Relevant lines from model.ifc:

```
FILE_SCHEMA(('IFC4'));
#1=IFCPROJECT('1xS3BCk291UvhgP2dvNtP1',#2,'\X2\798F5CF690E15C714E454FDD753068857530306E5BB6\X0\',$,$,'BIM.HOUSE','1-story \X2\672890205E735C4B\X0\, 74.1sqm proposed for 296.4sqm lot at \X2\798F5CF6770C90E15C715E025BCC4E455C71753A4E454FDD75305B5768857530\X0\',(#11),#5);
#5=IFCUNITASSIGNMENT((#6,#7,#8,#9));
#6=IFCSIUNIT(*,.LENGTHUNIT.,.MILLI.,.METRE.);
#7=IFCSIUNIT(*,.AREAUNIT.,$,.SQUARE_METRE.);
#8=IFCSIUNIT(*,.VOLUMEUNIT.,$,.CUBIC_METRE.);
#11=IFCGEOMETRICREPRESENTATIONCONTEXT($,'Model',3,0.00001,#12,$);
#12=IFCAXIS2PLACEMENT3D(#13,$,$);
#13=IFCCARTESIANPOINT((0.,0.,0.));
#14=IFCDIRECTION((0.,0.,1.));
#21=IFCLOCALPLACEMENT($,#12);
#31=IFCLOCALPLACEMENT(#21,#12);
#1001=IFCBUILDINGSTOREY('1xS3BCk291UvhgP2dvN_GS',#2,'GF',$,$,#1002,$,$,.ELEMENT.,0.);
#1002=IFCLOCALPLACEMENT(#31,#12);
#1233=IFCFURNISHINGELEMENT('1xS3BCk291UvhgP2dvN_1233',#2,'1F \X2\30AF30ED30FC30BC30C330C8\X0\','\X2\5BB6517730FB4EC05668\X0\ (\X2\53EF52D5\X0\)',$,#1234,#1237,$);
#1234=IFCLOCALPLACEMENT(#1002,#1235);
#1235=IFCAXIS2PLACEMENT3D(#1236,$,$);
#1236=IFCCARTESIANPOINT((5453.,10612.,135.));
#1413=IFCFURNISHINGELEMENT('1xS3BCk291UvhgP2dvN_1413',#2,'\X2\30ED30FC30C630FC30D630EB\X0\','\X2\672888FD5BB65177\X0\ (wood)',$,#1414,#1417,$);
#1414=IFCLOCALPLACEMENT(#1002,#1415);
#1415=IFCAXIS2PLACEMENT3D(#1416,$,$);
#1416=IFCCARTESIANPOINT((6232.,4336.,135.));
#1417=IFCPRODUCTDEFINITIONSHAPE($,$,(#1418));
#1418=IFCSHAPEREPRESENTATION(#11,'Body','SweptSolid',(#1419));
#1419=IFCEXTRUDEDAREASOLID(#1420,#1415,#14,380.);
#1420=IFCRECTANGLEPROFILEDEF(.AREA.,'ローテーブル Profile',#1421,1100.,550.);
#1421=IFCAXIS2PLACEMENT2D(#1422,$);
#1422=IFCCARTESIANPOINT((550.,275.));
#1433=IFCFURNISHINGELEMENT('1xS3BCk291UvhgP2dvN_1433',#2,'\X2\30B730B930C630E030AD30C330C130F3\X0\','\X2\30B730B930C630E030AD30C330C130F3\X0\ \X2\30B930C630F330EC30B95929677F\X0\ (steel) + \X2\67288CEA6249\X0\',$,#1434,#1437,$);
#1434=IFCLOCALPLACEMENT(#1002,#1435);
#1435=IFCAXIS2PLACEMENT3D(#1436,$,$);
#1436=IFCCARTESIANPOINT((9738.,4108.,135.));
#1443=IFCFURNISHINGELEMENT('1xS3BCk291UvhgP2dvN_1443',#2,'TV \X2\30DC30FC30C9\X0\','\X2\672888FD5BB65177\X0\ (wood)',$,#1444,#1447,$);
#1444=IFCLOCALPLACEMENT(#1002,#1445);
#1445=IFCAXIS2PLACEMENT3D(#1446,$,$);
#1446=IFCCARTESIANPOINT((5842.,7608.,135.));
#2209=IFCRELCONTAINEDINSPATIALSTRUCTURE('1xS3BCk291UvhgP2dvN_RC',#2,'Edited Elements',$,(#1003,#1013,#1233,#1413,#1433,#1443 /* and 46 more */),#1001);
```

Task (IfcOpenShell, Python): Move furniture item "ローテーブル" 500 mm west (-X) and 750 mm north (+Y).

```python
import ifcopenshell
import ifcopenshell.api.geometry
import ifcopenshell.util.placement

model = ifcopenshell.open("model.ifc")

item = model.by_guid("1xS3BCk291UvhgP2dvN_1413")
matrix = ifcopenshell.util.placement.get_local_placement(item.ObjectPlacement)
matrix[0, 3] -= 500.0
matrix[1, 3] += 750.0
ifcopenshell.api.geometry.edit_object_placement(model, product=item, matrix=matrix, is_si=False)

print(ifcopenshell.util.placement.get_local_placement(item.ObjectPlacement).round(3) + 0.0)

model.write("model-out.ifc")
```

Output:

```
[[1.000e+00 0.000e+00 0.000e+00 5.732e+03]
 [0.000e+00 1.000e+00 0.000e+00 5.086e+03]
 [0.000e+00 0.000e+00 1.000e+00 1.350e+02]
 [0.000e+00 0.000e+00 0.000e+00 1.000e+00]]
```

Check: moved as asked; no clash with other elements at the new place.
